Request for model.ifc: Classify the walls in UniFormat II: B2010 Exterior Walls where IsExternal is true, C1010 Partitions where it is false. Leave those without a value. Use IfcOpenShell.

First a look at what the model holds.

```python
import ifcopenshell
import ifcopenshell.util.element

model = ifcopenshell.open("model.ifc")
print(model.schema)
print("classifications:", [c.Name for c in model.by_type("IfcClassification")])
values = [ifcopenshell.util.element.get_pset(e, "Pset_WallCommon", "IsExternal") for e in model.by_type("IfcWall")]
for value in (True, False, None):
    print("IsExternal", value, values.count(value))
```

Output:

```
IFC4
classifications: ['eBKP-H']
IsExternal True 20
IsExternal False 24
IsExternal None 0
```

```python
import ifcopenshell
import ifcopenshell.api.classification
import ifcopenshell.util.element

model = ifcopenshell.open("model.ifc")

system = ifcopenshell.api.classification.add_classification(model, classification="UniFormat II")

walls = model.by_type("IfcWall")
external = {e: ifcopenshell.util.element.get_pset(e, "Pset_WallCommon", "IsExternal") for e in walls}
for flag, code, name in ((True, "B2010", "Exterior Walls"), (False, "C1010", "Partitions")):
    products = [e for e in walls if external[e] is flag]
    ifcopenshell.api.classification.add_reference(
        model, products=products, classification=system, identification=code, name=name
    )
    print(code, len(products))

model.write("model_rev.ifc")
```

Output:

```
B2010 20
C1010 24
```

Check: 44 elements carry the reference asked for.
